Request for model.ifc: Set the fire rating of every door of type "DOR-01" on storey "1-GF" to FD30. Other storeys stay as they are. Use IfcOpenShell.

First a look at what the model holds.

```python
import ifcopenshell
import ifcopenshell.util.element

model = ifcopenshell.open("model.ifc")
print(model.schema)
storey = next(s for s in model.by_type("IfcBuildingStorey") if s.Name == "1-GF")
doors = [e for e in ifcopenshell.util.element.get_decomposition(storey) if e.is_a("IfcDoor")]
seen = {}
for e in doors:
    element_type = ifcopenshell.util.element.get_type(e)
    key = (element_type.Name if element_type != e and element_type else None, ifcopenshell.util.element.get_pset(e, "Pset_DoorCommon", "FireRating"))
    seen[key] = seen.get(key, 0) + 1
for (name, value), count in sorted(seen.items(), key=str):
    print(count, "x", name, "|", value)
```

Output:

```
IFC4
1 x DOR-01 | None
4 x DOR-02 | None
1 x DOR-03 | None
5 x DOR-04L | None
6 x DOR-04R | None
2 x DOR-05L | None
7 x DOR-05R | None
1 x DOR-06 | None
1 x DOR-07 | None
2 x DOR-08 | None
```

```python
import ifcopenshell
import ifcopenshell.api.pset
import ifcopenshell.util.element

model = ifcopenshell.open("model.ifc")

storey = next(s for s in model.by_type("IfcBuildingStorey") if s.Name == "1-GF")
doors = [e for e in ifcopenshell.util.element.get_decomposition(storey) if e.is_a("IfcDoor")]

count = 0
for e in doors:
    element_type = ifcopenshell.util.element.get_type(e)
    if element_type in (None, e) or element_type.Name != "DOR-01":
        continue
    # add_pset returns the element's existing set when there is one.
    pset = ifcopenshell.api.pset.add_pset(model, product=e, name="Pset_DoorCommon")
    ifcopenshell.api.pset.edit_pset(model, pset=pset, properties={"FireRating": "FD30"})
    count += 1

print(count, "doors updated")

model.write("model_rev.ifc")
```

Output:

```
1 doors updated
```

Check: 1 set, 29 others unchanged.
